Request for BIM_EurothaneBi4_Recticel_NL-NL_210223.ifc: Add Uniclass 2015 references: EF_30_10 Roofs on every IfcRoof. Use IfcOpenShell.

First a look at what the model holds.

```python
import ifcopenshell

model = ifcopenshell.open("BIM_EurothaneBi4_Recticel_NL-NL_210223.ifc")
print(model.schema)
print("classifications:", [c.Name for c in model.by_type("IfcClassification")])
for ifc_class in ("IfcDoor", "IfcRoof", "IfcStair", "IfcWall", "IfcWindow"):
    print(ifc_class, len(model.by_type(ifc_class)))
```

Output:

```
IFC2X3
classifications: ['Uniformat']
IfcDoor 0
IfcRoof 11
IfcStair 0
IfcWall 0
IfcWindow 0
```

```python
import ifcopenshell
import ifcopenshell.api.classification

model = ifcopenshell.open("BIM_EurothaneBi4_Recticel_NL-NL_210223.ifc")

# IFC2X3 requires Source and Edition and has no link from the project to the system.
system = model.create_entity("IfcClassification", Source="NBS", Edition="2015", Name="Uniclass 2015")

codes = {
    "IfcRoof": ("EF_30_10", "Roofs"),
}
for ifc_class, (code, name) in codes.items():
    products = model.by_type(ifc_class)
    ifcopenshell.api.classification.add_reference(
        model, products=products, classification=system, identification=code, name=name
    )
    print(code, len(products))

model.write("BIM_EurothaneBi4_Recticel_NL-NL_210223_updated.ifc")
```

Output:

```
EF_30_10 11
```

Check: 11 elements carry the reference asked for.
